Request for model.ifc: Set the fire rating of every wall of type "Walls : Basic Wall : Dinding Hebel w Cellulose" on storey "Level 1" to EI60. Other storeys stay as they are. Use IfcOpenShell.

First a look at what the model holds.

```python
import ifcopenshell
import ifcopenshell.util.element

model = ifcopenshell.open("model.ifc")
print(model.schema)
storey = next(s for s in model.by_type("IfcBuildingStorey") if s.Name == "Level 1")
walls = [e for e in ifcopenshell.util.element.get_decomposition(storey) if e.is_a("IfcWall")]
seen = {}
for e in walls:
    element_type = ifcopenshell.util.element.get_type(e)
    key = (element_type.Name if element_type != e and element_type else None, ifcopenshell.util.element.get_pset(e, "Pset_WallCommon", "FireRating"))
    seen[key] = seen.get(key, 0) + 1
for (name, value), count in sorted(seen.items(), key=str):
    print(count, "x", name, "|", value)
```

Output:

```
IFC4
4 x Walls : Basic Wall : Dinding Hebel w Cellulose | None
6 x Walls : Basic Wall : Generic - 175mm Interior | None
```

```python
import ifcopenshell
import ifcopenshell.api.pset
import ifcopenshell.util.element

model = ifcopenshell.open("model.ifc")

storey = next(s for s in model.by_type("IfcBuildingStorey") if s.Name == "Level 1")
walls = [e for e in ifcopenshell.util.element.get_decomposition(storey) if e.is_a("IfcWall")]

count = 0
for e in walls:
    element_type = ifcopenshell.util.element.get_type(e)
    if element_type in (None, e) or element_type.Name != "Walls : Basic Wall : Dinding Hebel w Cellulose":
        continue
    # add_pset returns the element's existing set when there is one.
    pset = ifcopenshell.api.pset.add_pset(model, product=e, name="Pset_WallCommon")
    ifcopenshell.api.pset.edit_pset(model, pset=pset, properties={"FireRating": "EI60"})
    count += 1

print(count, "walls updated")

model.write("model_v2.ifc")
```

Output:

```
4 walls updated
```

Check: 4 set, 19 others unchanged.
